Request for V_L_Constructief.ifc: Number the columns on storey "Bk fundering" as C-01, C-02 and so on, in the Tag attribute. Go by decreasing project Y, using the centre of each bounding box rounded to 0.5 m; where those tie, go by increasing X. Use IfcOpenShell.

First a look at what the model holds.

```python
import ifcopenshell
import ifcopenshell.util.element
import ifcopenshell.util.placement

model = ifcopenshell.open("V_L_Constructief.ifc")
print(model.schema)
storey = next(s for s in model.by_type("IfcBuildingStorey") if s.Name == "Bk fundering")
columns = [e for e in ifcopenshell.util.element.get_decomposition(storey) if e.is_a("IfcColumn")]
for e in sorted(columns, key=lambda e: e.id()):
    origin = ifcopenshell.util.placement.get_local_placement(e.ObjectPlacement)[:3, 3]
    print(e.id(), e.Tag, e.Name, origin.round(2) + 0.0, sep=" | ")
```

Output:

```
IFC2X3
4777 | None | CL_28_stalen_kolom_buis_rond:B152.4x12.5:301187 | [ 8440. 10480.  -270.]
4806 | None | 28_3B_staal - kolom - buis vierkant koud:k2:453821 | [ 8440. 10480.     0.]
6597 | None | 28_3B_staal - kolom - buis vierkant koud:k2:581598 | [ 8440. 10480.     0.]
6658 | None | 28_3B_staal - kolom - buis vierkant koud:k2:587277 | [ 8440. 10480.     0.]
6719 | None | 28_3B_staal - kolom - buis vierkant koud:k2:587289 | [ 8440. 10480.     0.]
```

```python
import ifcopenshell
import ifcopenshell.geom
import ifcopenshell.util.element
import ifcopenshell.util.shape

model = ifcopenshell.open("V_L_Constructief.ifc")
settings = ifcopenshell.geom.settings()
settings.set("use-world-coords", True)


def centre(element):
    shape = ifcopenshell.geom.create_shape(settings, element)
    return ifcopenshell.util.shape.get_bbox_centroid(shape.geometry)


storey = next(s for s in model.by_type("IfcBuildingStorey") if s.Name == "Bk fundering")
columns = [e for e in ifcopenshell.util.element.get_decomposition(storey) if e.is_a("IfcColumn")]

# Insertion points can sit at a corner or the storey origin, so sort by the geometry (in metres).
centres = {e: centre(e) for e in columns}
columns.sort(key=lambda e: (-round(centres[e][1] / 0.5), centres[e][0]))

for i, e in enumerate(columns, start=1):
    number = f"C-{i:02d}"
    e.Tag = number
    print(e.id(), number)

model.write("V_L_Constructief-out.ifc")
```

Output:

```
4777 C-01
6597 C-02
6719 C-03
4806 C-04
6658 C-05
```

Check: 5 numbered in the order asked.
